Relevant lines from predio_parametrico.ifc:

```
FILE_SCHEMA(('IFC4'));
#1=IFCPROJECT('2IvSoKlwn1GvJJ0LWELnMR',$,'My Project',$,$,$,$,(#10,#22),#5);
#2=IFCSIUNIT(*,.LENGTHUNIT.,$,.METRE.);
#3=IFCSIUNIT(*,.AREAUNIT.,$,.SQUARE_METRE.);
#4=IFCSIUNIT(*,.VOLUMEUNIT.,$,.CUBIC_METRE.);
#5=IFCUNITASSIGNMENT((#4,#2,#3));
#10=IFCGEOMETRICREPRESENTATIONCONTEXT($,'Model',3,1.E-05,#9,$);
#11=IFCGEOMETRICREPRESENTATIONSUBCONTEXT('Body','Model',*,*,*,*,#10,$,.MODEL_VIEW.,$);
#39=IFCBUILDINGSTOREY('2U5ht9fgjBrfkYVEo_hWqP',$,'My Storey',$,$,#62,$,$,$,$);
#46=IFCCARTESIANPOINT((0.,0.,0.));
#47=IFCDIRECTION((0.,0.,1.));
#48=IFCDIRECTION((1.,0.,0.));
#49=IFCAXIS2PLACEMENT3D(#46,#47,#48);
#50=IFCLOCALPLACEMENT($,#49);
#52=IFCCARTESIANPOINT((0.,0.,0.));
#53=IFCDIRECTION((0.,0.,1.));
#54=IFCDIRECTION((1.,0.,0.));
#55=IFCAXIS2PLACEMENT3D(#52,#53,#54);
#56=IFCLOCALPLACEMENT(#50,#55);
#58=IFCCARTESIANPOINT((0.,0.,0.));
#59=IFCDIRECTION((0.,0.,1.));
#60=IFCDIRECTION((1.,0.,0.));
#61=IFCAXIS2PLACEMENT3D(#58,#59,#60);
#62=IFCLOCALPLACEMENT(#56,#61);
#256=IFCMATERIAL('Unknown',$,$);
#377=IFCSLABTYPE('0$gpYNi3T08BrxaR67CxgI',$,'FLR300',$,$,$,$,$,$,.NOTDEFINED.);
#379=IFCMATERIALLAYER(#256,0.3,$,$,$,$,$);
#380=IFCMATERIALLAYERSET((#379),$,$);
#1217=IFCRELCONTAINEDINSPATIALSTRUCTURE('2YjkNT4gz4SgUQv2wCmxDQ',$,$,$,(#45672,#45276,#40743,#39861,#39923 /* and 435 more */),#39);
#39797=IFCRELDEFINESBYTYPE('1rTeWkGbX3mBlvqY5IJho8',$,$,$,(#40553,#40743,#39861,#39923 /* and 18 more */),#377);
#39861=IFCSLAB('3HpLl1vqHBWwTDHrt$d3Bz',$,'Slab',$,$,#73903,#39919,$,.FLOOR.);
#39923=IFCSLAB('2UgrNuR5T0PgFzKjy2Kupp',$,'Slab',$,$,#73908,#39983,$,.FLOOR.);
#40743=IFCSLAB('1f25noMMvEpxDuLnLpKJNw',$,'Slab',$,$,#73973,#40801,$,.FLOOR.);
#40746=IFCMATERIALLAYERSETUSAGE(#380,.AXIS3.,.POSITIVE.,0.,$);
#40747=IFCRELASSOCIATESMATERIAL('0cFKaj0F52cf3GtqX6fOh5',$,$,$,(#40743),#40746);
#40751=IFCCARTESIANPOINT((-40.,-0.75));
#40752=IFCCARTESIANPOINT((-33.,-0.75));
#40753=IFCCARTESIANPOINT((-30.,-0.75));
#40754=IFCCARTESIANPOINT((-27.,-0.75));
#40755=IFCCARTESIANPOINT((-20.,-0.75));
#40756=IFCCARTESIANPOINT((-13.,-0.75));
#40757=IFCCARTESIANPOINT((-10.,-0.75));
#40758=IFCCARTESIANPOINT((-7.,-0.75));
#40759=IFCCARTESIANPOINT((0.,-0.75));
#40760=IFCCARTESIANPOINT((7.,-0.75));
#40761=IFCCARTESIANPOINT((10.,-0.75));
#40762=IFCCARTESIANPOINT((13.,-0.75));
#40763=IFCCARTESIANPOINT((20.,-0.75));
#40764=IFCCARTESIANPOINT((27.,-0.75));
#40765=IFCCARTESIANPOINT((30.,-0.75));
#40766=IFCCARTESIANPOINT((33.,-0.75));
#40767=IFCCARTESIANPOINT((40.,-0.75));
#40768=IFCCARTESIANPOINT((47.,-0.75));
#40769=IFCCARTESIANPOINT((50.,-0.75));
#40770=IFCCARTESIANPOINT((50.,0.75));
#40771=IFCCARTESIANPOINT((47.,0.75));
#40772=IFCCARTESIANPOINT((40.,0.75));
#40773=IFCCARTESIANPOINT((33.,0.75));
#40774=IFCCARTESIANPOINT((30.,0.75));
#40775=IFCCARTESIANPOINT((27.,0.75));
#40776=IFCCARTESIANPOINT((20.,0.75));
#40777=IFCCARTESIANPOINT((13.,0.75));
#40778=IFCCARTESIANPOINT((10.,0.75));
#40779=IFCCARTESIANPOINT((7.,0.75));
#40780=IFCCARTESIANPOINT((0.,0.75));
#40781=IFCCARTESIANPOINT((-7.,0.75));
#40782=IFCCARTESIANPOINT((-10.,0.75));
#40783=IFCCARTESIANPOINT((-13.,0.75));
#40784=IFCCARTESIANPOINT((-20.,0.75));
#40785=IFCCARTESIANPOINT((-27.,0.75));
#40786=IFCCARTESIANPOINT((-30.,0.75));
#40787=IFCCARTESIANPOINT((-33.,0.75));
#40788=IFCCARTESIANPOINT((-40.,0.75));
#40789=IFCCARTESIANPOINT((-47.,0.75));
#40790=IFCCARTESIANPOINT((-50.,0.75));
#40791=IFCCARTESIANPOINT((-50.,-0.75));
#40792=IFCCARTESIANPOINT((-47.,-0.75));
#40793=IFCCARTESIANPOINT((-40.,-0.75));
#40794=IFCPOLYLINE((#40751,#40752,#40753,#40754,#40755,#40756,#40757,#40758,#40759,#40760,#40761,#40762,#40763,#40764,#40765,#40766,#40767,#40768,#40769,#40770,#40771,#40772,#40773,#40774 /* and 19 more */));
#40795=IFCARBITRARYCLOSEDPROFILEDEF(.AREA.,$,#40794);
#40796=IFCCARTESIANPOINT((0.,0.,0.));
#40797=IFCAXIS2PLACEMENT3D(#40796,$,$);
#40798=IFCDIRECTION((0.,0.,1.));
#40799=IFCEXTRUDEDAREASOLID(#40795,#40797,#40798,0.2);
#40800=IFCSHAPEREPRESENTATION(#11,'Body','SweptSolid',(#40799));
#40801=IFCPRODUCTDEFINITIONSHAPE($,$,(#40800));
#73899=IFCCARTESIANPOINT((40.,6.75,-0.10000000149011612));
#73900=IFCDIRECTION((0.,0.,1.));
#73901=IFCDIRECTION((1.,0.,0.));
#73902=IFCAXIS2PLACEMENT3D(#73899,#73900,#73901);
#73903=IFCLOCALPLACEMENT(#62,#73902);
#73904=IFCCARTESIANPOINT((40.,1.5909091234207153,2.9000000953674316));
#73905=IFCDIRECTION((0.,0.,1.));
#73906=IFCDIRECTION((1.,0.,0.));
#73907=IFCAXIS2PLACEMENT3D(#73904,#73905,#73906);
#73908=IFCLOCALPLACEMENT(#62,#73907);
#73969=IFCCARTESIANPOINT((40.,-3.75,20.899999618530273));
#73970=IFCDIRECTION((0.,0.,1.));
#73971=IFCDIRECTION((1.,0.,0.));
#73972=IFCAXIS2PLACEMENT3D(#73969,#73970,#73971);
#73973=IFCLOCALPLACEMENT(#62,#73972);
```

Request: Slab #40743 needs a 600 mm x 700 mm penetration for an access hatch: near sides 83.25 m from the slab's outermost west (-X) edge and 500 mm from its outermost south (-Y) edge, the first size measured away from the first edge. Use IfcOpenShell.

```python
import numpy as np
import ifcopenshell
import ifcopenshell.api.feature
import ifcopenshell.api.geometry
import ifcopenshell.api.root
import ifcopenshell.geom
import ifcopenshell.util.placement
import ifcopenshell.util.representation
import ifcopenshell.util.shape
import ifcopenshell.util.unit

model = ifcopenshell.open("predio_parametrico.ifc")
unit_scale = ifcopenshell.util.unit.calculate_unit_scale(model)
settings = ifcopenshell.geom.settings()


def volume(element):
    """Net volume in cubic metres, openings subtracted."""
    shape = ifcopenshell.geom.create_shape(settings, element)
    return ifcopenshell.util.shape.get_volume(shape.geometry)


slab = model.by_guid("1f25noMMvEpxDuLnLpKJNw")
before = volume(slab)

# Extent in the slab's own axes, in metres. The edges named are its -X and -Y sides.
slab_shape = ifcopenshell.geom.create_shape(settings, slab)
vertices = ifcopenshell.util.shape.get_vertices(slab_shape.geometry)
x_min, y_min, bottom = vertices.min(axis=0)
top = vertices[:, 2].max()

opening = ifcopenshell.api.root.create_entity(model, ifc_class="IfcOpeningElement", name="Access hatch opening", predefined_type="OPENING")
context = ifcopenshell.util.representation.get_context(model, "Model", "Body", "MODEL_VIEW")
width, depth = 0.6, 0.7
outline = [(0.0, 0.0), (width, 0.0), (width, depth), (0.0, depth), (0.0, 0.0)]
# Overshoot both faces by 50 mm so the cut is clean.
shape = ifcopenshell.api.geometry.add_slab_representation(
    model, context=context, depth=top - bottom + 0.1, polyline=outline
)
ifcopenshell.api.geometry.assign_representation(model, product=opening, representation=shape)

matrix = ifcopenshell.util.placement.get_local_placement(slab.ObjectPlacement)
matrix[:, 3] = matrix @ np.append(np.array([x_min + 83.25, y_min + 0.5, bottom - 0.05]) / unit_scale, 1.0)
ifcopenshell.api.geometry.edit_object_placement(model, product=opening, matrix=matrix, is_si=False)
ifcopenshell.api.feature.add_feature(model, feature=opening, element=slab)

after = volume(slab)

print(f"slab volume {before:.3f} -> {after:.3f} m3")

model.write("predio_parametrico-out.ifc")
```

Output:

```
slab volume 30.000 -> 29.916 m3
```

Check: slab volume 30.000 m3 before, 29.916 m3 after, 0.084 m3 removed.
